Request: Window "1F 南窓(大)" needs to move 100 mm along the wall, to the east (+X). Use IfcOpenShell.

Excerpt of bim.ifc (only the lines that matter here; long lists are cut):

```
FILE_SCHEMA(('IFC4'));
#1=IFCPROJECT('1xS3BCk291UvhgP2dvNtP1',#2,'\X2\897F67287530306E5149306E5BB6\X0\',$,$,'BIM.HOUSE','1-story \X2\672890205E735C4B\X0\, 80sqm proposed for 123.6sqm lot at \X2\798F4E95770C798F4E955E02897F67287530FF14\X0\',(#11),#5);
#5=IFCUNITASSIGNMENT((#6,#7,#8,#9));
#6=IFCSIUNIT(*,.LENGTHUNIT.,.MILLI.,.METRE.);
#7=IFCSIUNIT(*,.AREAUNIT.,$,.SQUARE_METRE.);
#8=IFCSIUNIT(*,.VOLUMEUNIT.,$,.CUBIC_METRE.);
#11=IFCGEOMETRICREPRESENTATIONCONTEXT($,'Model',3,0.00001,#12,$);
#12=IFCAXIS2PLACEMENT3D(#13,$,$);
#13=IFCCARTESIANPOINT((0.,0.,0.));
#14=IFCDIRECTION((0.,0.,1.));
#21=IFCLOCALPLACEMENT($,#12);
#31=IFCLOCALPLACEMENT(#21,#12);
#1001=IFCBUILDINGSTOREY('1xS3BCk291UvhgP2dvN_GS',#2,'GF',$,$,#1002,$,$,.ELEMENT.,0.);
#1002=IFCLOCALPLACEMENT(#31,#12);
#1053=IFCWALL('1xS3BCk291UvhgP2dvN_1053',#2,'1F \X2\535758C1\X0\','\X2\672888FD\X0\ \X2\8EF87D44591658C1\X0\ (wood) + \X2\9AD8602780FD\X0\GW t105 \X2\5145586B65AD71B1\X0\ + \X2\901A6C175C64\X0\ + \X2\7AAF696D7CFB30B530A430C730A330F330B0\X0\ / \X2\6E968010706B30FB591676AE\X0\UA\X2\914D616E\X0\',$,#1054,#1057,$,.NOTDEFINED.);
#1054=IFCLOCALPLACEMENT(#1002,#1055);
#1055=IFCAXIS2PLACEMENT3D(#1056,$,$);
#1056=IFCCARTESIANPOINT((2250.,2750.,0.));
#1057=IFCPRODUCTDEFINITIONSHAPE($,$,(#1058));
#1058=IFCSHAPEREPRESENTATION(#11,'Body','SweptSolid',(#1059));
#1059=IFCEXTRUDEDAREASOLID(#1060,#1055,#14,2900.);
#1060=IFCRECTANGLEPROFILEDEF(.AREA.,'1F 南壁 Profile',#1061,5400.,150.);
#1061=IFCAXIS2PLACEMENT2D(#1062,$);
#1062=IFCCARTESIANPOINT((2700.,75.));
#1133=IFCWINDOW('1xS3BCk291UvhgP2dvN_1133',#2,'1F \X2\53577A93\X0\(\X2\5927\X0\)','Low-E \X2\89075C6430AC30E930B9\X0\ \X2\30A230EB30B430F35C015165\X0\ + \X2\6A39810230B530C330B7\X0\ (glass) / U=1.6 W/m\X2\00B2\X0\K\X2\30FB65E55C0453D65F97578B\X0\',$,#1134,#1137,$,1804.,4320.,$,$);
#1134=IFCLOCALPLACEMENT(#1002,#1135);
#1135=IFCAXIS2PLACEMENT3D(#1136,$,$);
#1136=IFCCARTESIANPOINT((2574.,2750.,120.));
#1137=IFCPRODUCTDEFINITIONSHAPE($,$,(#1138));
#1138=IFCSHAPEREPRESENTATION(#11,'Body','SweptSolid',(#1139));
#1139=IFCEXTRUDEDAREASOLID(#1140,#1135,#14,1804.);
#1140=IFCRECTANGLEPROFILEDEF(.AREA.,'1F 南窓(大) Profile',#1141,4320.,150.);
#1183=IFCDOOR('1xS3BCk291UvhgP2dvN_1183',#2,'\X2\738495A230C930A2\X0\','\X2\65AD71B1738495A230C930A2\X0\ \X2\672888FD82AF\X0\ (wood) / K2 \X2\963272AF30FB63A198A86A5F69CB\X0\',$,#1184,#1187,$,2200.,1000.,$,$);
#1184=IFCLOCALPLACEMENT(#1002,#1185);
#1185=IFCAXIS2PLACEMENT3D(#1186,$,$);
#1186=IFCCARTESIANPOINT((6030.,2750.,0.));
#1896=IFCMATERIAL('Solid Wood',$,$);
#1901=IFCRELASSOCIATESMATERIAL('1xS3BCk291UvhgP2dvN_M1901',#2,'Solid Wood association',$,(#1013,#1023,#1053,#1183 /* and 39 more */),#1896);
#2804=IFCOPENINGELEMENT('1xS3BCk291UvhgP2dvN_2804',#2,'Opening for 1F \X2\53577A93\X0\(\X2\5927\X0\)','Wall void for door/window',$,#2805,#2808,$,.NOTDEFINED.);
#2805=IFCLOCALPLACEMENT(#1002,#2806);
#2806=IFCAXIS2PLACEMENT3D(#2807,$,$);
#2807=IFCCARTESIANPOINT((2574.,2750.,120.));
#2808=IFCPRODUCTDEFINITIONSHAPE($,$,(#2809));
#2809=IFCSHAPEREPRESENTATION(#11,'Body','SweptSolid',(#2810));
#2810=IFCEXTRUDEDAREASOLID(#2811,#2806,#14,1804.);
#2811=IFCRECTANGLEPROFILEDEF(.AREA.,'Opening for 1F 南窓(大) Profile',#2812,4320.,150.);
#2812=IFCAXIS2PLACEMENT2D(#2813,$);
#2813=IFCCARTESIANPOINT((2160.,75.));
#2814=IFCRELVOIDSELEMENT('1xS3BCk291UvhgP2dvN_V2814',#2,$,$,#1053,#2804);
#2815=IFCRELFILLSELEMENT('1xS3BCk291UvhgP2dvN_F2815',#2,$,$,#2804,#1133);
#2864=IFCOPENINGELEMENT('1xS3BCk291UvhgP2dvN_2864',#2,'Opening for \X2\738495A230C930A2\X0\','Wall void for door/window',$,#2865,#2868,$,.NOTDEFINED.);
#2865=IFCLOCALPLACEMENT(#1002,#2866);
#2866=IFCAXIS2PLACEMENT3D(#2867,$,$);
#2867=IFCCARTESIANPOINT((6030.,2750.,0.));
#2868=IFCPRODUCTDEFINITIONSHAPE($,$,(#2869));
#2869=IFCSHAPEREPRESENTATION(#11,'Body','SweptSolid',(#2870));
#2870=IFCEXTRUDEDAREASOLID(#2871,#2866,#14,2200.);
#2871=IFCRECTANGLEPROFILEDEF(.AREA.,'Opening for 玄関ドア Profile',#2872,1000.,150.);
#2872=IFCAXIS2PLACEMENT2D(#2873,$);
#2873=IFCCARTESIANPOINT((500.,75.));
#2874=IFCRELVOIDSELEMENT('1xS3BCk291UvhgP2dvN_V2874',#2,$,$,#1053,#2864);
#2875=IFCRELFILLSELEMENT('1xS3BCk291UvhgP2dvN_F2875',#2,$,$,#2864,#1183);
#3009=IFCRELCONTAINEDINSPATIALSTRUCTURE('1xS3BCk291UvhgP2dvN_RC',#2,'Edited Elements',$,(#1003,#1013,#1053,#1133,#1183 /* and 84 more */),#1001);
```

```python
import ifcopenshell
import ifcopenshell.api.geometry
import ifcopenshell.util.placement
import ifcopenshell.util.unit

model = ifcopenshell.open("bim.ifc")
unit_scale = ifcopenshell.util.unit.calculate_unit_scale(model)

window = model.by_id(1133)
opening = window.FillsVoids[0].RelatingOpeningElement
wall = opening.VoidsElements[0].RelatingBuildingElement

wall_matrix = ifcopenshell.util.placement.get_local_placement(wall.ObjectPlacement)
shift = wall_matrix[:3, 0] * 0.1 / unit_scale
before = ifcopenshell.util.placement.get_local_placement(window.ObjectPlacement)[:3, 3].copy()

# The window is not placed relative to its opening, so move both.
for product in (opening, window):
    matrix = ifcopenshell.util.placement.get_local_placement(product.ObjectPlacement)
    matrix[:3, 3] += shift
    ifcopenshell.api.geometry.edit_object_placement(model, product=product, matrix=matrix, is_si=False)

after = ifcopenshell.util.placement.get_local_placement(window.ObjectPlacement)[:3, 3]
print("window moved by", (after - before).round(3) + 0.0)

model.write("bim_rev.ifc")
```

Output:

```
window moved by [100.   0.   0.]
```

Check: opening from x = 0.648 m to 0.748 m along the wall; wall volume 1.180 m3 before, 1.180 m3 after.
